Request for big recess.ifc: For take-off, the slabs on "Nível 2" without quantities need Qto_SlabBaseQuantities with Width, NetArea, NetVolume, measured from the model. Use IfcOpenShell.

First a look at what the model holds.

```python
import ifcopenshell
import ifcopenshell.util.element
import ifcopenshell.util.unit

model = ifcopenshell.open("big recess.ifc")
print(model.schema)
for unit_type in ("LENGTHUNIT", "AREAUNIT", "VOLUMEUNIT"):
    print(unit_type, ifcopenshell.util.unit.calculate_unit_scale(model, unit_type))
storey = next(s for s in model.by_type("IfcBuildingStorey") if s.Name == "Nível 2")
slabs = [e for e in ifcopenshell.util.element.get_decomposition(storey) if e.is_a("IfcSlab")]
for e in sorted(slabs, key=lambda e: e.id()):
    print(e.id(), e.is_a(), e.Name, list(ifcopenshell.util.element.get_psets(e, qtos_only=True)), sep=" | ")
```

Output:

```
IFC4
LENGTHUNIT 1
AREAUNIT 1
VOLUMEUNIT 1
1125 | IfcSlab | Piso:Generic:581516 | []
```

```python
import ifcopenshell
import ifcopenshell.api.pset
import ifcopenshell.geom
import ifcopenshell.util.element
import ifcopenshell.util.shape
import ifcopenshell.util.unit

model = ifcopenshell.open("big recess.ifc")
unit_scale = ifcopenshell.util.unit.calculate_unit_scale(model)
area_scale = ifcopenshell.util.unit.calculate_unit_scale(model, "AREAUNIT")
volume_scale = ifcopenshell.util.unit.calculate_unit_scale(model, "VOLUMEUNIT")
settings = ifcopenshell.geom.settings()

storey = next(s for s in model.by_type("IfcBuildingStorey") if s.Name == "Nível 2")
slabs = [e for e in ifcopenshell.util.element.get_decomposition(storey) if e.is_a("IfcSlab")]

for e in sorted(slabs, key=lambda e: e.id()):
    if ifcopenshell.util.element.get_psets(e, qtos_only=True, should_inherit=False):
        continue
    # Geometry comes back in metres, in the element's own axes.
    shape = ifcopenshell.geom.create_shape(settings, e)
    values = {
        "Width": ifcopenshell.util.shape.get_z(shape.geometry) / unit_scale,
        "NetArea": ifcopenshell.util.shape.get_footprint_area(shape.geometry) / area_scale,
        "NetVolume": ifcopenshell.util.shape.get_volume(shape.geometry) / volume_scale,
    }
    qto = ifcopenshell.api.pset.add_qto(model, product=e, name="Qto_SlabBaseQuantities")
    ifcopenshell.api.pset.edit_qto(model, qto=qto, properties=values)
    print(e.id(), {k: round(v, 3) for k, v in values.items()})

model.write("big recess_edited.ifc")
```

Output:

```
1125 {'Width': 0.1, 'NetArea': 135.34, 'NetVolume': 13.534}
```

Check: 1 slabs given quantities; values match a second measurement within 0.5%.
